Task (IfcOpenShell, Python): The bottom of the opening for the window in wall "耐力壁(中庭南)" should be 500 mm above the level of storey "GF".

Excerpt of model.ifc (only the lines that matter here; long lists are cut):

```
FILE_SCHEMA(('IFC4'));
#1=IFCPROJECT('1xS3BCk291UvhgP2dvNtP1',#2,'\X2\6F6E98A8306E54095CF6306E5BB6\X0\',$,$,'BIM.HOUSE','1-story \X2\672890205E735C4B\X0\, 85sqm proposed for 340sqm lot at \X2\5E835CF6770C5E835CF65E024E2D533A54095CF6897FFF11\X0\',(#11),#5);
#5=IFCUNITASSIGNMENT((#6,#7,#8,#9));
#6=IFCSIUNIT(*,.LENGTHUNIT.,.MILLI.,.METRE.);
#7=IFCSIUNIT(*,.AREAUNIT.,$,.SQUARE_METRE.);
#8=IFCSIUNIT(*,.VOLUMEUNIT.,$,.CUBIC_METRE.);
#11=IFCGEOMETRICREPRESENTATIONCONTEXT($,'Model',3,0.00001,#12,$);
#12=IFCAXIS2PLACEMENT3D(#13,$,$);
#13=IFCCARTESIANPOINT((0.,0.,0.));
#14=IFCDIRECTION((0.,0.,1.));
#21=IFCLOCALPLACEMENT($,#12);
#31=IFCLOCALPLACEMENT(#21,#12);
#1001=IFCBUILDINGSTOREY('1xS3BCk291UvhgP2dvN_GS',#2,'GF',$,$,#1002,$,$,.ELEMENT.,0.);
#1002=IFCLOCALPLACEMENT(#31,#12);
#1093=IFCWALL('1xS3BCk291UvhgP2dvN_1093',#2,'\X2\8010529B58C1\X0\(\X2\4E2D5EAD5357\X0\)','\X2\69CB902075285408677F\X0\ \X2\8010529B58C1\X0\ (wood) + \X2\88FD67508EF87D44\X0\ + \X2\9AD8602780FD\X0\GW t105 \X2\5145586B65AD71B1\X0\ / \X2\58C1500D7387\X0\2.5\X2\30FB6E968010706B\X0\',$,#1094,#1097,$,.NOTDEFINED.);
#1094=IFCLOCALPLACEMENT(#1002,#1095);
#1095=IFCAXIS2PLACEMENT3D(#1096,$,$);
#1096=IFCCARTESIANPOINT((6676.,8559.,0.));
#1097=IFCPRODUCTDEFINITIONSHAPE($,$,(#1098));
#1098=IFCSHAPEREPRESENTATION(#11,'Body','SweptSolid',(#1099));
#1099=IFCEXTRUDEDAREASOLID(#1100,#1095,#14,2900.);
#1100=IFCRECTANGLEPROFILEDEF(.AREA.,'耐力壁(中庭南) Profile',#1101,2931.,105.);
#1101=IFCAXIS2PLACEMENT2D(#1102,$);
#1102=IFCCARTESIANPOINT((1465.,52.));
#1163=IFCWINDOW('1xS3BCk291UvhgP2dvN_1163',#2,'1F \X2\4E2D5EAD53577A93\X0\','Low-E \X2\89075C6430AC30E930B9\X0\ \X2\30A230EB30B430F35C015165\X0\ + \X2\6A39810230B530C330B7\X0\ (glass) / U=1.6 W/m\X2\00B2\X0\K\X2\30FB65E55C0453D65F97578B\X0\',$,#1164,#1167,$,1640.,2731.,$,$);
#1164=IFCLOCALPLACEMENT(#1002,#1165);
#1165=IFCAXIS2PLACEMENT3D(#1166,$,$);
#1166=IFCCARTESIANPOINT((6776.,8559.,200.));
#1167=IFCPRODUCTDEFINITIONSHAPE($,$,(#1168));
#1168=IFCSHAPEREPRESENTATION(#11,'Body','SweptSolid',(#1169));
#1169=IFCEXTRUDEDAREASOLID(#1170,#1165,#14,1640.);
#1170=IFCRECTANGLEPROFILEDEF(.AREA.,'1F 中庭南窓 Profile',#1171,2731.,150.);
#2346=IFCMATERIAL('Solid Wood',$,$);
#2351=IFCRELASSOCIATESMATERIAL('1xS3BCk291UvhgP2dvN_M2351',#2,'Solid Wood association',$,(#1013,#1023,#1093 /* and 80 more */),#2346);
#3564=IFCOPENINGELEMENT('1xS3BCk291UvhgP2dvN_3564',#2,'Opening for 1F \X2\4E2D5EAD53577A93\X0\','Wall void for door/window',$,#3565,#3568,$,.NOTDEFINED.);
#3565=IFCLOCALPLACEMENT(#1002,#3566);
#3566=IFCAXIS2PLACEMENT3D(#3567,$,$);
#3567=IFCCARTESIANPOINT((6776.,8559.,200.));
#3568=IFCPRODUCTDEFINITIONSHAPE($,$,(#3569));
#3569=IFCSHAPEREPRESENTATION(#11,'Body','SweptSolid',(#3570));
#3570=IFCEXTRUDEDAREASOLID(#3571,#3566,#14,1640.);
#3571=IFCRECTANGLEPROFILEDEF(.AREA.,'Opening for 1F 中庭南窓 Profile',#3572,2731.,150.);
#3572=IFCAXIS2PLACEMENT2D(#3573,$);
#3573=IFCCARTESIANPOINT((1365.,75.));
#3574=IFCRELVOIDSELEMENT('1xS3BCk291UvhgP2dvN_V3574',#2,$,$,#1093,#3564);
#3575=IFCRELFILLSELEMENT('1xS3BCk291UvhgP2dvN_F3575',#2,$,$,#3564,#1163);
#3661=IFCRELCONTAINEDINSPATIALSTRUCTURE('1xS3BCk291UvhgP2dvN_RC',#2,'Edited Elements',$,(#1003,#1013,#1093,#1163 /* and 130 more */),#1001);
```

```python
import numpy as np
import ifcopenshell
import ifcopenshell.api.geometry
import ifcopenshell.geom
import ifcopenshell.util.element
import ifcopenshell.util.placement
import ifcopenshell.util.shape
import ifcopenshell.util.unit

model = ifcopenshell.open("model.ifc")
unit_scale = ifcopenshell.util.unit.calculate_unit_scale(model)

window = model.by_id(1163)
opening = window.FillsVoids[0].RelatingOpeningElement
storey = ifcopenshell.util.element.get_container(window, ifc_class="IfcBuildingStorey")
level = ifcopenshell.util.placement.get_local_placement(storey.ObjectPlacement)[2, 3]

# The opening's origin need not be at the sill, so measure its lowest point.
shape = ifcopenshell.geom.create_shape(ifcopenshell.geom.settings(), opening)
bottom = ifcopenshell.util.shape.get_shape_bottom_elevation(shape, shape.geometry) / unit_scale
dz = level + 0.5 / unit_scale - bottom

shift = np.array([0.0, 0.0, dz])
# The window is not placed relative to its opening, so move both.
for product in (opening, window):
    matrix = ifcopenshell.util.placement.get_local_placement(product.ObjectPlacement)
    matrix[:3, 3] += shift
    ifcopenshell.api.geometry.edit_object_placement(model, product=product, matrix=matrix, is_si=False)

print(f"moved by {dz * unit_scale:+.3f} m")

model.write("model_rev.ifc")
```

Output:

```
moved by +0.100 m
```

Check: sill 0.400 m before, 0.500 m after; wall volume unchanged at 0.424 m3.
